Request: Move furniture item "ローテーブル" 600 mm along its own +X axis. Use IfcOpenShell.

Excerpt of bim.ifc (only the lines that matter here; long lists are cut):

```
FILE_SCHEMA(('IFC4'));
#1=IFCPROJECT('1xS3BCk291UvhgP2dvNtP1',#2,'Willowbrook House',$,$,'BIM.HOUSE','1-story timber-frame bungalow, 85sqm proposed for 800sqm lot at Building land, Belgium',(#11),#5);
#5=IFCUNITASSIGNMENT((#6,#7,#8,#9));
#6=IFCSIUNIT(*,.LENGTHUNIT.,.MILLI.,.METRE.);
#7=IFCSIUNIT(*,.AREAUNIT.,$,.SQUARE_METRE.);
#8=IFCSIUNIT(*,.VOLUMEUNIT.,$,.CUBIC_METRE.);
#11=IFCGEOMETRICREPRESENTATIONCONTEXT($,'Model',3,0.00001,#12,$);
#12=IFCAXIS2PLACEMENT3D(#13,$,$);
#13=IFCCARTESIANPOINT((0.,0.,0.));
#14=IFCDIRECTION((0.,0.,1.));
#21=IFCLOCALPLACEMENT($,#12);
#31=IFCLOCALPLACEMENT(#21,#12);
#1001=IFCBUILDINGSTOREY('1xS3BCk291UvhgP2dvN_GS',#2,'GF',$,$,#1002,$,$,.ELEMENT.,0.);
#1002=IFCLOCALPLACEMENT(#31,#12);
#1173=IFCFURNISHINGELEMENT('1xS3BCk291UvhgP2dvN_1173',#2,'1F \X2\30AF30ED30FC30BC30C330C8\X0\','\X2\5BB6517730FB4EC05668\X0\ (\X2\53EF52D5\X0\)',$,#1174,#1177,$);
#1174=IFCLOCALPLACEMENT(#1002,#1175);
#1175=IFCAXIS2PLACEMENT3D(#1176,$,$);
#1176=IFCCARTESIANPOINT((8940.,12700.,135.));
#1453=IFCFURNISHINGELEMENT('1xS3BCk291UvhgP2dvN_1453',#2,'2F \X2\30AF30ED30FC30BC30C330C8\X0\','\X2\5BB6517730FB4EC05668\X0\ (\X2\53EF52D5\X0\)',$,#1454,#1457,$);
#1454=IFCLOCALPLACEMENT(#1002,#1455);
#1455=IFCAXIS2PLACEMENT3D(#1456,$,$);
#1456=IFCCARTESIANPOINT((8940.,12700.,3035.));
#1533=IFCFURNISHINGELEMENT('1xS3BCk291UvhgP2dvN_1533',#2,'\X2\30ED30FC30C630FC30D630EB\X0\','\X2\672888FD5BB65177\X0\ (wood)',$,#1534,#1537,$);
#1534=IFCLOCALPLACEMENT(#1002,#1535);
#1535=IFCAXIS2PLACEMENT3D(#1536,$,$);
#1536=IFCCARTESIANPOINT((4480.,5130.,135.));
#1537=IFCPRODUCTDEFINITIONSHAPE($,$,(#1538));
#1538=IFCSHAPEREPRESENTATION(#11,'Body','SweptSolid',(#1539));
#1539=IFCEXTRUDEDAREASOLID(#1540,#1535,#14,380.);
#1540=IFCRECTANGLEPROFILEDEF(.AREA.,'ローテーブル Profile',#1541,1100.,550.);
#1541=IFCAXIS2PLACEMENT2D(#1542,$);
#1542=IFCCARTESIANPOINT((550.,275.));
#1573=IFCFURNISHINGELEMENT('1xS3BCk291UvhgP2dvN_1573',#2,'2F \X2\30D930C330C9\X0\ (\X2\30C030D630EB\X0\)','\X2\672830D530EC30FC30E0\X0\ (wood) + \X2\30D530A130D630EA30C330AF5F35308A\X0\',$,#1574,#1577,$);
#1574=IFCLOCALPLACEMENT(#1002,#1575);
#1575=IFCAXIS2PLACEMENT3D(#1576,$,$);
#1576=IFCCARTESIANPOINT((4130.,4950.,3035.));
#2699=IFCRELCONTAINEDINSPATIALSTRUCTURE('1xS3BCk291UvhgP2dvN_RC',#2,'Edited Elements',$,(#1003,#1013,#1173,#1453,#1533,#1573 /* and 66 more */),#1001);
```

```python
import ifcopenshell
import ifcopenshell.api.geometry
import ifcopenshell.util.placement

model = ifcopenshell.open("bim.ifc")

item = model.by_guid("1xS3BCk291UvhgP2dvN_1533")
matrix = ifcopenshell.util.placement.get_local_placement(item.ObjectPlacement)
matrix[:3, 3] += matrix[:3, 0] * 600.0
ifcopenshell.api.geometry.edit_object_placement(model, product=item, matrix=matrix, is_si=False)

print(ifcopenshell.util.placement.get_local_placement(item.ObjectPlacement).round(3) + 0.0)

model.write("bim_edited.ifc")
```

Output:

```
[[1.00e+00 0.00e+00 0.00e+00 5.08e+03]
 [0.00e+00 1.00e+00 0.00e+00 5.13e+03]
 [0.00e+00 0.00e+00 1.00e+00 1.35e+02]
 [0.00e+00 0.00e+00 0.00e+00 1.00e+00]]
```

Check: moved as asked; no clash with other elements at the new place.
